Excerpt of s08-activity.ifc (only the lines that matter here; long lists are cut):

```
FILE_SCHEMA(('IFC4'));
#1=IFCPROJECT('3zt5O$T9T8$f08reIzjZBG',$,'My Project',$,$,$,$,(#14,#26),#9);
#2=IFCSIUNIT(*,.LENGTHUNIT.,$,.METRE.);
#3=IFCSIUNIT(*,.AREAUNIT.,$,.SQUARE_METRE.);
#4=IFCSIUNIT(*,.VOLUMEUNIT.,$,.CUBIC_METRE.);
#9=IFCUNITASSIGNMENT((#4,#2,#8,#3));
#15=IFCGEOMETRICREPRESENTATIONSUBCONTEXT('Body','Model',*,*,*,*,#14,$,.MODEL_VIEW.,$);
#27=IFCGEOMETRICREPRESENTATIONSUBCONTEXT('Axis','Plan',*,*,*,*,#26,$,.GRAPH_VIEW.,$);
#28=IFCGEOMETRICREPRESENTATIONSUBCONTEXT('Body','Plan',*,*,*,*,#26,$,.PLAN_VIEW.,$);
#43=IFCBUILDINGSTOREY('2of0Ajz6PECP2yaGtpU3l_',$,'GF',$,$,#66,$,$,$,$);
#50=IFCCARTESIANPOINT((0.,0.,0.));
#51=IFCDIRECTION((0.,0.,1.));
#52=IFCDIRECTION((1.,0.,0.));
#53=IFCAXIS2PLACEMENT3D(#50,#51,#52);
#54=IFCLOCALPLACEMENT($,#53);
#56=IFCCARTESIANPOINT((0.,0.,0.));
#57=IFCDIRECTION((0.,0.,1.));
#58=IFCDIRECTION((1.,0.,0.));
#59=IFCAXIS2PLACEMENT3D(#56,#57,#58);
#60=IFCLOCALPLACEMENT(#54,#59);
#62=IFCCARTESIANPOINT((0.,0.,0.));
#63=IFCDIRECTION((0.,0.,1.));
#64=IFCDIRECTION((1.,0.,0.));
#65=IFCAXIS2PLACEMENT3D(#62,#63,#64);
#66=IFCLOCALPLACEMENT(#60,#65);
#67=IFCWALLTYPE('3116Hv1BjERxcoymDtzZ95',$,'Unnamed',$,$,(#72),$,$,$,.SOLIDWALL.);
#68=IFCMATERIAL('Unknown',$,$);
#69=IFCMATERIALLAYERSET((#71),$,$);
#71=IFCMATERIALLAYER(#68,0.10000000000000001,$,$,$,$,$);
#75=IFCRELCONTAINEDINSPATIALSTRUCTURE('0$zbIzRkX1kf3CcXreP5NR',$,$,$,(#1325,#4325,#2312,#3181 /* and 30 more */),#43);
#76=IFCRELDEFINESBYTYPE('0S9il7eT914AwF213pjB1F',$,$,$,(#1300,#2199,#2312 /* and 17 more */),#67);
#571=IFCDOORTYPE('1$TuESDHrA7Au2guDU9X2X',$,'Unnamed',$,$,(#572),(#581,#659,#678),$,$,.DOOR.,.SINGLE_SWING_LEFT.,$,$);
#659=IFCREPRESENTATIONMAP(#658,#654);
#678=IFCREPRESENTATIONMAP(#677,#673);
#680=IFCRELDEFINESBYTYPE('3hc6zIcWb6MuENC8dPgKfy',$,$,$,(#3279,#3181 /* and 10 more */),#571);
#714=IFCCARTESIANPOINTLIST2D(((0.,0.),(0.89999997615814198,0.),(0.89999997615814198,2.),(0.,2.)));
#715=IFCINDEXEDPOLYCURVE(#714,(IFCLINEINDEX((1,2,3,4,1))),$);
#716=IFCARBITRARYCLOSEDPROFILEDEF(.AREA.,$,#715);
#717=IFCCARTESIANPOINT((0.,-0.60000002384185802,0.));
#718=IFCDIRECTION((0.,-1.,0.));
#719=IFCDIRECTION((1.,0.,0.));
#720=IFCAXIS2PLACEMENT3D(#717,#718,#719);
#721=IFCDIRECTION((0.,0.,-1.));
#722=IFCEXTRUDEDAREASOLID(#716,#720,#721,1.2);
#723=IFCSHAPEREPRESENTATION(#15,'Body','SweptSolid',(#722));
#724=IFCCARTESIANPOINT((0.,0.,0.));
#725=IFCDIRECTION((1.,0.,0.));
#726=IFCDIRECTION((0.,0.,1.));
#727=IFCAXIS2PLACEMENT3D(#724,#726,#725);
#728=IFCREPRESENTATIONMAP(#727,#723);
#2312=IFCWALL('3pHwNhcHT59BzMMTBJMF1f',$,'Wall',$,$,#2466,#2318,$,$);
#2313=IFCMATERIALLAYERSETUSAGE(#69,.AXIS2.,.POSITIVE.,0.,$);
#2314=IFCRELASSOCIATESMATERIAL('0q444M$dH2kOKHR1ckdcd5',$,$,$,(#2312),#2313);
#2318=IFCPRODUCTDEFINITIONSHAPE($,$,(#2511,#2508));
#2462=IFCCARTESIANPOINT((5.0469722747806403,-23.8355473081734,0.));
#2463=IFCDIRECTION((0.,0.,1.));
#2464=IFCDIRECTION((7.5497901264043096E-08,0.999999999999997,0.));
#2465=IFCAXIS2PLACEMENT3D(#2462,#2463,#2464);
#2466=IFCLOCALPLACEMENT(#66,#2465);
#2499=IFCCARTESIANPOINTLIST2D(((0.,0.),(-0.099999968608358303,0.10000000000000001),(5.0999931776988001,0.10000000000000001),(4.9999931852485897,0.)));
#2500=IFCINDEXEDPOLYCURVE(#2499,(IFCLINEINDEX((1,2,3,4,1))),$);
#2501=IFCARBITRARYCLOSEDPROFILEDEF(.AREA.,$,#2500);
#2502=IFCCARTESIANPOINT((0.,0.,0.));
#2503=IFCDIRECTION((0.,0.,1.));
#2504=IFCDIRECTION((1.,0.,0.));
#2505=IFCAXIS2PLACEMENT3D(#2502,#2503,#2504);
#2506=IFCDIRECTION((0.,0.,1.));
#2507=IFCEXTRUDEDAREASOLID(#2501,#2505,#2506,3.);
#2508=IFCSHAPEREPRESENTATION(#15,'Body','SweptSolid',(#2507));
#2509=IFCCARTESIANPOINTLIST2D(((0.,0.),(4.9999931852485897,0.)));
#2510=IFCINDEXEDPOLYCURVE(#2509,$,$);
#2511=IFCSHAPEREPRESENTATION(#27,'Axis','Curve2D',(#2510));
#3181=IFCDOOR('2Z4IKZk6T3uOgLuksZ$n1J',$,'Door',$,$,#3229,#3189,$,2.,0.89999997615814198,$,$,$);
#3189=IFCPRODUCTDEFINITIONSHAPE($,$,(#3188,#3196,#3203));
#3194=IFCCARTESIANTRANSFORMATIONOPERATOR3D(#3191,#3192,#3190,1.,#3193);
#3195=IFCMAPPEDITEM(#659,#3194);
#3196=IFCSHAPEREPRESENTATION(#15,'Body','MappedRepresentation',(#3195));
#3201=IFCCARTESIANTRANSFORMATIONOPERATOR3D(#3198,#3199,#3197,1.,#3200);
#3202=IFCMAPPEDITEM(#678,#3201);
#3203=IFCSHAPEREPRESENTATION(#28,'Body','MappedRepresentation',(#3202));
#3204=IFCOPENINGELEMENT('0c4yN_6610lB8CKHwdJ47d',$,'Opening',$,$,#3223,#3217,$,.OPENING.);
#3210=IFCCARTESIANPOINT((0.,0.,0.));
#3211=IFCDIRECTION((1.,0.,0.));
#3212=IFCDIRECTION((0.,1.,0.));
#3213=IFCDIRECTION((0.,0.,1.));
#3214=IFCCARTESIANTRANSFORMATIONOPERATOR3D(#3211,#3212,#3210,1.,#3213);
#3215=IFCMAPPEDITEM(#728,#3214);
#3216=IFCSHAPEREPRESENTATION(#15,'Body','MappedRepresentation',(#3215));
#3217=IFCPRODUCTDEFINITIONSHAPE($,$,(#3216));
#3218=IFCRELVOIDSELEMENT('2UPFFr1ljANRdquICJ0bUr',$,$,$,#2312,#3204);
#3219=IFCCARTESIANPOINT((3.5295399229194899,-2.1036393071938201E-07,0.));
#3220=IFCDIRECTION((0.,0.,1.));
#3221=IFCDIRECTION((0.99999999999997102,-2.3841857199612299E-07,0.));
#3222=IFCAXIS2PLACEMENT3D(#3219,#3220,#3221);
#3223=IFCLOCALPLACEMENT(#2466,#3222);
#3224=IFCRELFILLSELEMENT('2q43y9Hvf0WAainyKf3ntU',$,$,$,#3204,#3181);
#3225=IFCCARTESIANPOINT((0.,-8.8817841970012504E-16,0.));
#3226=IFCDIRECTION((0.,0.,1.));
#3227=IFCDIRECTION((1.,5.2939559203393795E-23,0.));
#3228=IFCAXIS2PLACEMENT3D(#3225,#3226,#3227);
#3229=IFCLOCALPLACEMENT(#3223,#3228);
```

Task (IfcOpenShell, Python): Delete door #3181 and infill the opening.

```python
import ifcopenshell
import ifcopenshell.api.feature
import ifcopenshell.api.root
import ifcopenshell.geom
import ifcopenshell.util.shape

model = ifcopenshell.open("s08-activity.ifc")
settings = ifcopenshell.geom.settings()


def volume(element):
    """Net volume in cubic metres, openings subtracted."""
    shape = ifcopenshell.geom.create_shape(settings, element)
    return ifcopenshell.util.shape.get_volume(shape.geometry)


door = model.by_guid("2Z4IKZk6T3uOgLuksZ$n1J")
opening = door.FillsVoids[0].RelatingOpeningElement
wall = opening.VoidsElements[0].RelatingBuildingElement
before = volume(wall)

ifcopenshell.api.root.remove_product(model, product=door)
ifcopenshell.api.feature.remove_feature(model, feature=opening)

after = volume(wall)

print(f"wall volume {before:.3f} -> {after:.3f} m3")

model.write("s08-activity-out.ifc")
```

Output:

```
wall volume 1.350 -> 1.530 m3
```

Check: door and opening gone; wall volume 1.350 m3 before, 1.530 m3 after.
